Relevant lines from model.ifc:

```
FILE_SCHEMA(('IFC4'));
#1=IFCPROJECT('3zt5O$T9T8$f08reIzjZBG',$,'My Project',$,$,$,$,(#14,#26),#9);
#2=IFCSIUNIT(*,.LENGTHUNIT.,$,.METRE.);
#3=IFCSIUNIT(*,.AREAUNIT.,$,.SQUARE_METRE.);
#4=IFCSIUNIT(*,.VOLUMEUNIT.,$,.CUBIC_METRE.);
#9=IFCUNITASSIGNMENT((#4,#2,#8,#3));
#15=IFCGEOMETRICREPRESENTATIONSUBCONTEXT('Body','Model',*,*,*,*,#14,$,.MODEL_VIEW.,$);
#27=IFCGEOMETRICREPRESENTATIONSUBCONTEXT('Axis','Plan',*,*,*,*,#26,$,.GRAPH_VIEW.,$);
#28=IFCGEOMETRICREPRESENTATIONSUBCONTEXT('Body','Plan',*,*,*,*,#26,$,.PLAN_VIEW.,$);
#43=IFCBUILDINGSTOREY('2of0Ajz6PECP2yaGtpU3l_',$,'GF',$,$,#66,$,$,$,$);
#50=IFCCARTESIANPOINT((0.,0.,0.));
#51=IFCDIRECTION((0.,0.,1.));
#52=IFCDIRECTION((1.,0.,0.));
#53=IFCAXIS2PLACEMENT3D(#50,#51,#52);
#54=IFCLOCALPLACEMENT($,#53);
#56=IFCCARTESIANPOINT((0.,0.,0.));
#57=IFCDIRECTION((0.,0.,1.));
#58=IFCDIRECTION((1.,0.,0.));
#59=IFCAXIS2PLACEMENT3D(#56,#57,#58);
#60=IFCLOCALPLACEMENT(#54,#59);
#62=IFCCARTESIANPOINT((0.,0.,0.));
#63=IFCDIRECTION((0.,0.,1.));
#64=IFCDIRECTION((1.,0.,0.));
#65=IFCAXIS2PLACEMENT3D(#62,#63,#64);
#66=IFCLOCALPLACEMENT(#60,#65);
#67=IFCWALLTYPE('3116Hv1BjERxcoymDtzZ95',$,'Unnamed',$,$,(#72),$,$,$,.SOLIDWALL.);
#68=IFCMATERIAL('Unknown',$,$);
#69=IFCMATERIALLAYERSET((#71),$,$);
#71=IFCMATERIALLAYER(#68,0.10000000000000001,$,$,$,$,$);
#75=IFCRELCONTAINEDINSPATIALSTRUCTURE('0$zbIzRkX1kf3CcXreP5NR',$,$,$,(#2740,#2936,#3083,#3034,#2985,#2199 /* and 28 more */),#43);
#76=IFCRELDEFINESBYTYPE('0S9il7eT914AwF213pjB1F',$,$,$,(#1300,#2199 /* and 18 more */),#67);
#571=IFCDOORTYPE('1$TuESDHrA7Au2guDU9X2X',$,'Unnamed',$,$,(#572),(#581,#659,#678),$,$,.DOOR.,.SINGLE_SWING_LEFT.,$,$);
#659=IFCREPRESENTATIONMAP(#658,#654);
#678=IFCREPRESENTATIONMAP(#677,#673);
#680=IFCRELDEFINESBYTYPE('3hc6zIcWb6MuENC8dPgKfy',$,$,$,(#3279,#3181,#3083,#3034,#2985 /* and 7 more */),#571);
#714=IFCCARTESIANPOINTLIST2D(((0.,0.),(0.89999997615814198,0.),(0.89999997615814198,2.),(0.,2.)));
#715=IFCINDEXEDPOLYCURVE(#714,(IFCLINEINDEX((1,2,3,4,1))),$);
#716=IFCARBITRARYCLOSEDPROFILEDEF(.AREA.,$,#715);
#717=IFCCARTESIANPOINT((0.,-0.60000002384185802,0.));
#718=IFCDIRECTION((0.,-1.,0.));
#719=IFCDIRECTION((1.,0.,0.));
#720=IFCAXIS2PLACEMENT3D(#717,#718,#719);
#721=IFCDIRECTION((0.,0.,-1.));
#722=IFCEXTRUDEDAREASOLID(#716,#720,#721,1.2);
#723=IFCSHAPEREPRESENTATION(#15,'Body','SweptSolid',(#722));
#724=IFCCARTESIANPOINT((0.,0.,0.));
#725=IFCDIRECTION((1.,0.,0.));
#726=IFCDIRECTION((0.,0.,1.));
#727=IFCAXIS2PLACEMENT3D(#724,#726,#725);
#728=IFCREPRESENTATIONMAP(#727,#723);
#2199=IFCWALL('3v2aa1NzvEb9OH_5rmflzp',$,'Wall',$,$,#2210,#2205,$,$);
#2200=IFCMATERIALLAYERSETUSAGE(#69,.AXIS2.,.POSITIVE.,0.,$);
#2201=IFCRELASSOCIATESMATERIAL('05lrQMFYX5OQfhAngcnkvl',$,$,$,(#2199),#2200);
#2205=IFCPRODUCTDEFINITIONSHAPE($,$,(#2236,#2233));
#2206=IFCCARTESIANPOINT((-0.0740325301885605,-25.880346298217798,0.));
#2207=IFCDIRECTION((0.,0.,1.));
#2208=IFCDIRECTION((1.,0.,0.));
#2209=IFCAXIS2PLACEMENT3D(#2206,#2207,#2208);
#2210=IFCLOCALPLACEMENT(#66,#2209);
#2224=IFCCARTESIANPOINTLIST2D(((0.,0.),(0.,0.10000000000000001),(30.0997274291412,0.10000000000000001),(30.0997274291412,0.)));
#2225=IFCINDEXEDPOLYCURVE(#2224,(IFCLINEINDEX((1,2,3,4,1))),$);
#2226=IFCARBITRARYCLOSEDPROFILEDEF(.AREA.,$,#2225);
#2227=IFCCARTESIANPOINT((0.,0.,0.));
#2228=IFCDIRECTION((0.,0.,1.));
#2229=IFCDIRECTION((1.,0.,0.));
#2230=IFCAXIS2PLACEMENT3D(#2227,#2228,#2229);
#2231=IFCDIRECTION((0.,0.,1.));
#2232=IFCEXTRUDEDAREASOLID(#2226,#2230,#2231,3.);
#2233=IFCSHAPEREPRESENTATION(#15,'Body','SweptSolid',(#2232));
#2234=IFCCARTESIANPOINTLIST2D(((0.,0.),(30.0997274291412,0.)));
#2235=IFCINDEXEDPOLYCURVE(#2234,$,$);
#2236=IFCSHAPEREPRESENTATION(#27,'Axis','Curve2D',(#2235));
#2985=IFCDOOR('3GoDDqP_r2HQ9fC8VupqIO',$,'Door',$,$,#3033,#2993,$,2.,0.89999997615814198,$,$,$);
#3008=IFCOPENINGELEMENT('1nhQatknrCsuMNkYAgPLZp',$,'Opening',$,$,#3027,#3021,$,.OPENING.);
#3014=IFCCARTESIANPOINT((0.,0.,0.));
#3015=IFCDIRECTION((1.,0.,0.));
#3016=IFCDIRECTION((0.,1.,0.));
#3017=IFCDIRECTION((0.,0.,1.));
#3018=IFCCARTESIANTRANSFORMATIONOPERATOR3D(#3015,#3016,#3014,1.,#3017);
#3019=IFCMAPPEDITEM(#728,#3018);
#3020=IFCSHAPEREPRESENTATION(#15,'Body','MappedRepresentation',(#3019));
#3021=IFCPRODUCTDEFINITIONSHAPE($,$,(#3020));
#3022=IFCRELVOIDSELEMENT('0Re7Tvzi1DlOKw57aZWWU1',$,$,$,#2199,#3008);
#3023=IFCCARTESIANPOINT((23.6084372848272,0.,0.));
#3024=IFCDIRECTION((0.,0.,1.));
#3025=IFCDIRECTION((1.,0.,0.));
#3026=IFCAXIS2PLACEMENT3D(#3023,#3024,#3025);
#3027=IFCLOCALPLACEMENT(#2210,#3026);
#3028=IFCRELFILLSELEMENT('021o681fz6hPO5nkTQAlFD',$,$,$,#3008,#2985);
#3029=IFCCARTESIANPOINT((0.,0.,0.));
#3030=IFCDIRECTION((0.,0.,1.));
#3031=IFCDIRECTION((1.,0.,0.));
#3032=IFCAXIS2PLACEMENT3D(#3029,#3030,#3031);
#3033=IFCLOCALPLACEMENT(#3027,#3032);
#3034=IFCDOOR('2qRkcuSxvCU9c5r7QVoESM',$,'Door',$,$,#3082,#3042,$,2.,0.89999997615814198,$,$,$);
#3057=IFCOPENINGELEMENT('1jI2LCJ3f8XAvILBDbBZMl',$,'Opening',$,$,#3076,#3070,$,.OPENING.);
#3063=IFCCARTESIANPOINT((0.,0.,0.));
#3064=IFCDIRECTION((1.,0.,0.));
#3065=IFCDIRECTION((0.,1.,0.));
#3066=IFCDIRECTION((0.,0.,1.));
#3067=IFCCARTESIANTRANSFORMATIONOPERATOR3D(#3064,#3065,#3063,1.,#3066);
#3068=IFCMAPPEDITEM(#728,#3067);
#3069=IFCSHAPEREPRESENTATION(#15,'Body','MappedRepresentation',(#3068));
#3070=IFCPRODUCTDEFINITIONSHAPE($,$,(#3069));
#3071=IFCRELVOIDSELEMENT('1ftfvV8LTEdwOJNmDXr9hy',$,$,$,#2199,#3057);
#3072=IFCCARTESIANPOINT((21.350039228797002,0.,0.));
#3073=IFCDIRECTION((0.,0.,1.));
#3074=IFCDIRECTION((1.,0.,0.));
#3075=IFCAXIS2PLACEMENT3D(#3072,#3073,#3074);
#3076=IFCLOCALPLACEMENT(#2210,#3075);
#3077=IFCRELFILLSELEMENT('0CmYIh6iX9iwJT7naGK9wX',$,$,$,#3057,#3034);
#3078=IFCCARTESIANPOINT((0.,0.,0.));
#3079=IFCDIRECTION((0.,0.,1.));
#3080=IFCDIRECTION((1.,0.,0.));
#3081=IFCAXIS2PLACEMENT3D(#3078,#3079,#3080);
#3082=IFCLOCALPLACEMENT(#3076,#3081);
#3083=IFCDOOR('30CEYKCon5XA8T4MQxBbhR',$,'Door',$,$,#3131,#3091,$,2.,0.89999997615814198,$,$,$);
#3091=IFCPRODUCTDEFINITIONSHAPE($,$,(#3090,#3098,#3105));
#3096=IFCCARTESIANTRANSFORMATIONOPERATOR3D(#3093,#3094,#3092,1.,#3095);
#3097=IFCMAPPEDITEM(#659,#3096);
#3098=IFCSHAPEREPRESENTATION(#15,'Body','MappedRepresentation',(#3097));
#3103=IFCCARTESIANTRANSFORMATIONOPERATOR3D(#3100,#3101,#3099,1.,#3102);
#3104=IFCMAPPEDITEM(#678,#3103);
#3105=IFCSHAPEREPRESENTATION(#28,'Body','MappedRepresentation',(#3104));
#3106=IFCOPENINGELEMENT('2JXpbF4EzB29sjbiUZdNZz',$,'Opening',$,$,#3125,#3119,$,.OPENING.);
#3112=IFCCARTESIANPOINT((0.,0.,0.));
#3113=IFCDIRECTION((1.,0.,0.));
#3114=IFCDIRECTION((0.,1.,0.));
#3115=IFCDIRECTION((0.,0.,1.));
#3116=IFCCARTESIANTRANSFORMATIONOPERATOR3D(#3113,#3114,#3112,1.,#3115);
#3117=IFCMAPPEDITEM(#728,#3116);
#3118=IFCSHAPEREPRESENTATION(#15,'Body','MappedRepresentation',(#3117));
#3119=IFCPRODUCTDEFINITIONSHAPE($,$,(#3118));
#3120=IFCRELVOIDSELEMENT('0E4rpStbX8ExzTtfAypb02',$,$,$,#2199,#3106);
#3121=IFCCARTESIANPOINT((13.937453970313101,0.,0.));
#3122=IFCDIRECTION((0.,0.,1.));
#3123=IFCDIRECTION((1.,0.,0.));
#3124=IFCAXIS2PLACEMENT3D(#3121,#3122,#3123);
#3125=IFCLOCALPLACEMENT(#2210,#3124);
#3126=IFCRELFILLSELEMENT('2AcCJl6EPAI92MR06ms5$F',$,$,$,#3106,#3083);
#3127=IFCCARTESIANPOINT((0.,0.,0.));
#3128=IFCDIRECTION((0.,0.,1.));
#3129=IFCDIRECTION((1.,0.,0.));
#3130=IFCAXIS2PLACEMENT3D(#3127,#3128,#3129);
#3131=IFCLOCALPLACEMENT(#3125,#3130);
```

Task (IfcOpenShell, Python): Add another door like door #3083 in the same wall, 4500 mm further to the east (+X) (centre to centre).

```python
import ifcopenshell
import ifcopenshell.api.feature
import ifcopenshell.api.geometry
import ifcopenshell.api.root
import ifcopenshell.geom
import ifcopenshell.util.element
import ifcopenshell.util.placement
import ifcopenshell.util.shape

model = ifcopenshell.open("model.ifc")
settings = ifcopenshell.geom.settings()


def volume(element):
    """Net volume in cubic metres, openings subtracted."""
    shape = ifcopenshell.geom.create_shape(settings, element)
    return ifcopenshell.util.shape.get_volume(shape.geometry)


door = model.by_guid("30CEYKCon5XA8T4MQxBbhR")
opening = door.FillsVoids[0].RelatingOpeningElement
wall = opening.VoidsElements[0].RelatingBuildingElement
before = volume(wall)
shift = ifcopenshell.util.placement.get_local_placement(wall.ObjectPlacement)[:3, 0] * 4.5

# copy_class copies the void relationship, type, container and properties, but no geometry.
new_opening = ifcopenshell.api.root.copy_class(model, product=opening)
new_opening.Representation = ifcopenshell.util.element.copy_deep(
    model, opening.Representation, exclude=["IfcGeometricRepresentationContext", "IfcRepresentationMap"]
)
new_door = ifcopenshell.api.root.copy_class(model, product=door)
new_door.Representation = ifcopenshell.util.element.copy_deep(
    model, door.Representation, exclude=["IfcGeometricRepresentationContext", "IfcRepresentationMap"]
)
ifcopenshell.api.feature.add_filling(model, opening=new_opening, element=new_door)

for old, new in ((opening, new_opening), (door, new_door)):
    matrix = ifcopenshell.util.placement.get_local_placement(old.ObjectPlacement)
    matrix[:3, 3] += shift
    ifcopenshell.api.geometry.edit_object_placement(model, product=new, matrix=matrix, is_si=False)

after = volume(wall)

print(f"wall volume {before:.3f} -> {after:.3f} m3")

model.write("model_edited.ifc")
```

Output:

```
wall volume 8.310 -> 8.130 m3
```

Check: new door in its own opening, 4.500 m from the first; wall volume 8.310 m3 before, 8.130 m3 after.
